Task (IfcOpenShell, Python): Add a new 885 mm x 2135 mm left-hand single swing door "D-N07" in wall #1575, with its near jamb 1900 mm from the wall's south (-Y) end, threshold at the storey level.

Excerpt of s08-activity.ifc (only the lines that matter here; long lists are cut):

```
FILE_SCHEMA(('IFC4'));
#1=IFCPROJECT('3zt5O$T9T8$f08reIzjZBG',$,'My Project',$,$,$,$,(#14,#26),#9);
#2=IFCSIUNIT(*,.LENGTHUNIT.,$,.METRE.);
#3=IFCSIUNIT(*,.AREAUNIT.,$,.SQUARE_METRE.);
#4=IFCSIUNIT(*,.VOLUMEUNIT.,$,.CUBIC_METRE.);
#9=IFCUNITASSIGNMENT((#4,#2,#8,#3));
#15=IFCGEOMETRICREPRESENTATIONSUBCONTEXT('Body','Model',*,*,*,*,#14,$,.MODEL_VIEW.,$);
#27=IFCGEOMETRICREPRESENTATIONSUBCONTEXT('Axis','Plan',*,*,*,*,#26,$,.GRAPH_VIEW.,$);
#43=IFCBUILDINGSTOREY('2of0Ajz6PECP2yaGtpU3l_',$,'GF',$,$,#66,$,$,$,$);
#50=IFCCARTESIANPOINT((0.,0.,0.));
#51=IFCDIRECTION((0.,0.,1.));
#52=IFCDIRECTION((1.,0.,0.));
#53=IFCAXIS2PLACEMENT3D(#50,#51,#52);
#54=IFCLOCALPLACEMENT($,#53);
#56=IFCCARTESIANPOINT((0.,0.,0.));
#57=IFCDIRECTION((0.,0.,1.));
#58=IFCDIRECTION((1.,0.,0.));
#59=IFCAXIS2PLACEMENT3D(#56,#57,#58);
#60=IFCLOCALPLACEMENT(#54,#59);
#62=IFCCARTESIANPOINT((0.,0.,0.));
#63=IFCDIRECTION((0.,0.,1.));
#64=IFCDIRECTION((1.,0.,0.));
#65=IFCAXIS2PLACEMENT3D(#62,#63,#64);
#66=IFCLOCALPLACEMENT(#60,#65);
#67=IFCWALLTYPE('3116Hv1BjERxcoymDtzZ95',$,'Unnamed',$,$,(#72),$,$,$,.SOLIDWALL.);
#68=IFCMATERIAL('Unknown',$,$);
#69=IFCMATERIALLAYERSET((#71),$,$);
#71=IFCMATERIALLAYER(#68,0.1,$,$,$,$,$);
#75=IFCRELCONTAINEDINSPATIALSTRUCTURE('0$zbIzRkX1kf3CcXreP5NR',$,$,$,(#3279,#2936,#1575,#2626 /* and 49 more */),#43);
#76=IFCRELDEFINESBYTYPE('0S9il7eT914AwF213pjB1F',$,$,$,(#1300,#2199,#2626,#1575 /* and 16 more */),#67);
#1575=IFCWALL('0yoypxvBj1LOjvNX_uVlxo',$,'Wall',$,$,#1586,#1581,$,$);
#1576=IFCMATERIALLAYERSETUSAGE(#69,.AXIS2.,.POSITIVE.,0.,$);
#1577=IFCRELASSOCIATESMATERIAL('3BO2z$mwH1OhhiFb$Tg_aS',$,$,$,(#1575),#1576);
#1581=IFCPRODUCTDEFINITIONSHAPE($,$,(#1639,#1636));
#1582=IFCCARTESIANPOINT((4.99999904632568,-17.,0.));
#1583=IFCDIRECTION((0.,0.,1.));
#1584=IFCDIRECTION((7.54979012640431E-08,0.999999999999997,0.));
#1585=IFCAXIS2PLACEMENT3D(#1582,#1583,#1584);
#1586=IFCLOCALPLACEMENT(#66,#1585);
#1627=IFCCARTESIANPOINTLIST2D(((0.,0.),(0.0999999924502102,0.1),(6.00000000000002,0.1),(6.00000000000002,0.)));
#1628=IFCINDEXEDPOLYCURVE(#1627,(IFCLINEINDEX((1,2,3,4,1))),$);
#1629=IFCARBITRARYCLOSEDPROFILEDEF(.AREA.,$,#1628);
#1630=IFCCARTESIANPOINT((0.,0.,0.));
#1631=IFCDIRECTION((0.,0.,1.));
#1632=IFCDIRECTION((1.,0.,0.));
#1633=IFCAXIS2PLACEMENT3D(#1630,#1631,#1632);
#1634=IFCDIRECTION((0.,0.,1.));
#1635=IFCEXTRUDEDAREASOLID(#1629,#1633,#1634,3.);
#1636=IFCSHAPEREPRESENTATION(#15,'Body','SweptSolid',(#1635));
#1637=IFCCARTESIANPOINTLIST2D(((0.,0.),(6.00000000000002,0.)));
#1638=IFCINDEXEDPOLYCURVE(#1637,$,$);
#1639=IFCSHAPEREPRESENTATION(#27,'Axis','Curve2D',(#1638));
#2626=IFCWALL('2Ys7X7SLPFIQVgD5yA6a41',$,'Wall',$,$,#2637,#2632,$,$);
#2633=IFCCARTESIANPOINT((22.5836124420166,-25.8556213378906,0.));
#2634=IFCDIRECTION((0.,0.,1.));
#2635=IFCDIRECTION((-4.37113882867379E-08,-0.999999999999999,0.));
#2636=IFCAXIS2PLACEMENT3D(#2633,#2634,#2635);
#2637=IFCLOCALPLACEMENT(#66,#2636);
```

```python
import numpy as np
import ifcopenshell
import ifcopenshell.api.feature
import ifcopenshell.api.geometry
import ifcopenshell.api.root
import ifcopenshell.api.spatial
import ifcopenshell.geom
import ifcopenshell.util.element
import ifcopenshell.util.placement
import ifcopenshell.util.representation
import ifcopenshell.util.shape
import ifcopenshell.util.unit

model = ifcopenshell.open("s08-activity.ifc")
unit_scale = ifcopenshell.util.unit.calculate_unit_scale(model)
settings = ifcopenshell.geom.settings()


def volume(element):
    """Net volume in cubic metres, openings subtracted."""
    shape = ifcopenshell.geom.create_shape(settings, element)
    return ifcopenshell.util.shape.get_volume(shape.geometry)


wall = model.by_guid("0yoypxvBj1LOjvNX_uVlxo")
storey = ifcopenshell.util.element.get_container(wall, ifc_class="IfcBuildingStorey")
context = ifcopenshell.util.representation.get_context(model, "Model", "Body", "MODEL_VIEW")
before = volume(wall)

width, height, from_end, sill = 0.885, 2.135, 1.9, 0.0  # metres

# The wall runs along its own X axis, and the end named is its -X end.
wall_shape = ifcopenshell.geom.create_shape(settings, wall)
x, y, z = ifcopenshell.util.shape.get_vertices(wall_shape.geometry).T
start = x.min() + from_end
face, thickness = float(y.min()), float(y.max() - y.min())
wall_matrix = ifcopenshell.util.placement.get_local_placement(wall.ObjectPlacement)
level = ifcopenshell.util.placement.get_local_placement(storey.ObjectPlacement)[2, 3]


def in_wall(x, y):
    """Placement at x, y metres in the wall's axes, at sill height."""
    matrix = wall_matrix.copy()
    matrix[:, 3] = wall_matrix @ np.array([x / unit_scale, y / unit_scale, 0.0, 1.0])
    matrix[2, 3] = level + sill / unit_scale
    return matrix


# Opening: a box that overshoots both wall faces by 50 mm.
opening = ifcopenshell.api.root.create_entity(model, ifc_class="IfcOpeningElement", predefined_type="OPENING")
box = ifcopenshell.api.geometry.add_wall_representation(
    model, context=context, length=width, height=height, thickness=thickness + 0.1
)
ifcopenshell.api.geometry.assign_representation(model, product=opening, representation=box)
ifcopenshell.api.geometry.edit_object_placement(model, product=opening, matrix=in_wall(start, face - 0.05), is_si=False)
ifcopenshell.api.feature.add_feature(model, feature=opening, element=wall)

door = ifcopenshell.api.root.create_entity(model, ifc_class="IfcDoor", name="D-N07", predefined_type="DOOR")
door.OverallWidth, door.OverallHeight = width / unit_scale, height / unit_scale
door.OperationType = "SINGLE_SWING_LEFT"
body = ifcopenshell.api.geometry.add_door_representation(
    model,
    context=context,
    overall_width=door.OverallWidth,
    overall_height=door.OverallHeight,
    operation_type="SINGLE_SWING_LEFT",
    lining_properties={"LiningDepth": thickness / unit_scale, "ThresholdDepth": thickness / unit_scale},
)
ifcopenshell.api.geometry.assign_representation(model, product=door, representation=body)
ifcopenshell.api.spatial.assign_container(model, products=[door], relating_structure=storey)
ifcopenshell.api.feature.add_filling(model, opening=opening, element=door)

# The lining spans the wall, so the door starts at the wall face.
ifcopenshell.api.geometry.edit_object_placement(model, product=door, matrix=in_wall(start, face), is_si=False)

after = volume(wall)

print(f"wall volume {before:.3f} -> {after:.3f} m3")

model.write("s08-activity_v2.ifc")
```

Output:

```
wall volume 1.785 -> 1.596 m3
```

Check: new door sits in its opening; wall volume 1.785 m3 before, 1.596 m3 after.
